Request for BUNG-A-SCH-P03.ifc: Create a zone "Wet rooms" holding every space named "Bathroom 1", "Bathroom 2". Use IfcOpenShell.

First a look at what the model holds.

```python
import ifcopenshell

model = ifcopenshell.open("BUNG-A-SCH-P03.ifc")
print(model.schema)
seen = {}
for space in model.by_type("IfcSpace"):
    seen[space.LongName] = seen.get(space.LongName, 0) + 1
for name, count in sorted(seen.items(), key=str):
    print(count, "x", name)
print("zones:", [z.Name for z in model.by_type("IfcZone")][:20])
```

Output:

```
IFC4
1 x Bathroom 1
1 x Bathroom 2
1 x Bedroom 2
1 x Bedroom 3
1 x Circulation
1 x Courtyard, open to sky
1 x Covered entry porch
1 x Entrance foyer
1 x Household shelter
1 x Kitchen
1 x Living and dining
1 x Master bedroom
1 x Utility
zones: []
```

```python
import ifcopenshell
import ifcopenshell.api.group
import ifcopenshell.api.root

model = ifcopenshell.open("BUNG-A-SCH-P03.ifc")

names = {"Bathroom 1", "Bathroom 2"}
spaces = [s for s in model.by_type("IfcSpace") if s.LongName in names]

zone = ifcopenshell.api.root.create_entity(model, ifc_class="IfcZone", name="Wet rooms")
ifcopenshell.api.group.assign_group(model, products=spaces, group=zone)
print(len(spaces), "spaces in", zone.Name)

model.write("BUNG-A-SCH-P03-out.ifc")
```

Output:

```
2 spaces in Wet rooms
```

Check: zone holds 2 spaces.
